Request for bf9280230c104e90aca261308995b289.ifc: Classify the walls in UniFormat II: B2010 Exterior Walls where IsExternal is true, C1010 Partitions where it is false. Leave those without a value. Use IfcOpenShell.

First a look at what the model holds.

```python
import ifcopenshell
import ifcopenshell.util.element

model = ifcopenshell.open("bf9280230c104e90aca261308995b289.ifc")
print(model.schema)
print("classifications:", [c.Name for c in model.by_type("IfcClassification")])
values = [ifcopenshell.util.element.get_pset(e, "Pset_WallCommon", "IsExternal") for e in model.by_type("IfcWall")]
for value in (True, False, None):
    print("IsExternal", value, values.count(value))
```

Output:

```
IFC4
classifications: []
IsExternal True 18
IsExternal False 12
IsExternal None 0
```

```python
import ifcopenshell
import ifcopenshell.api.classification
import ifcopenshell.util.element

model = ifcopenshell.open("bf9280230c104e90aca261308995b289.ifc")

system = ifcopenshell.api.classification.add_classification(model, classification="UniFormat II")

walls = model.by_type("IfcWall")
external = {e: ifcopenshell.util.element.get_pset(e, "Pset_WallCommon", "IsExternal") for e in walls}
for flag, code, name in ((True, "B2010", "Exterior Walls"), (False, "C1010", "Partitions")):
    products = [e for e in walls if external[e] is flag]
    ifcopenshell.api.classification.add_reference(
        model, products=products, classification=system, identification=code, name=name
    )
    print(code, len(products))

model.write("bf9280230c104e90aca261308995b289_updated.ifc")
```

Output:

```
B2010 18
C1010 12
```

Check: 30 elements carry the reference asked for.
